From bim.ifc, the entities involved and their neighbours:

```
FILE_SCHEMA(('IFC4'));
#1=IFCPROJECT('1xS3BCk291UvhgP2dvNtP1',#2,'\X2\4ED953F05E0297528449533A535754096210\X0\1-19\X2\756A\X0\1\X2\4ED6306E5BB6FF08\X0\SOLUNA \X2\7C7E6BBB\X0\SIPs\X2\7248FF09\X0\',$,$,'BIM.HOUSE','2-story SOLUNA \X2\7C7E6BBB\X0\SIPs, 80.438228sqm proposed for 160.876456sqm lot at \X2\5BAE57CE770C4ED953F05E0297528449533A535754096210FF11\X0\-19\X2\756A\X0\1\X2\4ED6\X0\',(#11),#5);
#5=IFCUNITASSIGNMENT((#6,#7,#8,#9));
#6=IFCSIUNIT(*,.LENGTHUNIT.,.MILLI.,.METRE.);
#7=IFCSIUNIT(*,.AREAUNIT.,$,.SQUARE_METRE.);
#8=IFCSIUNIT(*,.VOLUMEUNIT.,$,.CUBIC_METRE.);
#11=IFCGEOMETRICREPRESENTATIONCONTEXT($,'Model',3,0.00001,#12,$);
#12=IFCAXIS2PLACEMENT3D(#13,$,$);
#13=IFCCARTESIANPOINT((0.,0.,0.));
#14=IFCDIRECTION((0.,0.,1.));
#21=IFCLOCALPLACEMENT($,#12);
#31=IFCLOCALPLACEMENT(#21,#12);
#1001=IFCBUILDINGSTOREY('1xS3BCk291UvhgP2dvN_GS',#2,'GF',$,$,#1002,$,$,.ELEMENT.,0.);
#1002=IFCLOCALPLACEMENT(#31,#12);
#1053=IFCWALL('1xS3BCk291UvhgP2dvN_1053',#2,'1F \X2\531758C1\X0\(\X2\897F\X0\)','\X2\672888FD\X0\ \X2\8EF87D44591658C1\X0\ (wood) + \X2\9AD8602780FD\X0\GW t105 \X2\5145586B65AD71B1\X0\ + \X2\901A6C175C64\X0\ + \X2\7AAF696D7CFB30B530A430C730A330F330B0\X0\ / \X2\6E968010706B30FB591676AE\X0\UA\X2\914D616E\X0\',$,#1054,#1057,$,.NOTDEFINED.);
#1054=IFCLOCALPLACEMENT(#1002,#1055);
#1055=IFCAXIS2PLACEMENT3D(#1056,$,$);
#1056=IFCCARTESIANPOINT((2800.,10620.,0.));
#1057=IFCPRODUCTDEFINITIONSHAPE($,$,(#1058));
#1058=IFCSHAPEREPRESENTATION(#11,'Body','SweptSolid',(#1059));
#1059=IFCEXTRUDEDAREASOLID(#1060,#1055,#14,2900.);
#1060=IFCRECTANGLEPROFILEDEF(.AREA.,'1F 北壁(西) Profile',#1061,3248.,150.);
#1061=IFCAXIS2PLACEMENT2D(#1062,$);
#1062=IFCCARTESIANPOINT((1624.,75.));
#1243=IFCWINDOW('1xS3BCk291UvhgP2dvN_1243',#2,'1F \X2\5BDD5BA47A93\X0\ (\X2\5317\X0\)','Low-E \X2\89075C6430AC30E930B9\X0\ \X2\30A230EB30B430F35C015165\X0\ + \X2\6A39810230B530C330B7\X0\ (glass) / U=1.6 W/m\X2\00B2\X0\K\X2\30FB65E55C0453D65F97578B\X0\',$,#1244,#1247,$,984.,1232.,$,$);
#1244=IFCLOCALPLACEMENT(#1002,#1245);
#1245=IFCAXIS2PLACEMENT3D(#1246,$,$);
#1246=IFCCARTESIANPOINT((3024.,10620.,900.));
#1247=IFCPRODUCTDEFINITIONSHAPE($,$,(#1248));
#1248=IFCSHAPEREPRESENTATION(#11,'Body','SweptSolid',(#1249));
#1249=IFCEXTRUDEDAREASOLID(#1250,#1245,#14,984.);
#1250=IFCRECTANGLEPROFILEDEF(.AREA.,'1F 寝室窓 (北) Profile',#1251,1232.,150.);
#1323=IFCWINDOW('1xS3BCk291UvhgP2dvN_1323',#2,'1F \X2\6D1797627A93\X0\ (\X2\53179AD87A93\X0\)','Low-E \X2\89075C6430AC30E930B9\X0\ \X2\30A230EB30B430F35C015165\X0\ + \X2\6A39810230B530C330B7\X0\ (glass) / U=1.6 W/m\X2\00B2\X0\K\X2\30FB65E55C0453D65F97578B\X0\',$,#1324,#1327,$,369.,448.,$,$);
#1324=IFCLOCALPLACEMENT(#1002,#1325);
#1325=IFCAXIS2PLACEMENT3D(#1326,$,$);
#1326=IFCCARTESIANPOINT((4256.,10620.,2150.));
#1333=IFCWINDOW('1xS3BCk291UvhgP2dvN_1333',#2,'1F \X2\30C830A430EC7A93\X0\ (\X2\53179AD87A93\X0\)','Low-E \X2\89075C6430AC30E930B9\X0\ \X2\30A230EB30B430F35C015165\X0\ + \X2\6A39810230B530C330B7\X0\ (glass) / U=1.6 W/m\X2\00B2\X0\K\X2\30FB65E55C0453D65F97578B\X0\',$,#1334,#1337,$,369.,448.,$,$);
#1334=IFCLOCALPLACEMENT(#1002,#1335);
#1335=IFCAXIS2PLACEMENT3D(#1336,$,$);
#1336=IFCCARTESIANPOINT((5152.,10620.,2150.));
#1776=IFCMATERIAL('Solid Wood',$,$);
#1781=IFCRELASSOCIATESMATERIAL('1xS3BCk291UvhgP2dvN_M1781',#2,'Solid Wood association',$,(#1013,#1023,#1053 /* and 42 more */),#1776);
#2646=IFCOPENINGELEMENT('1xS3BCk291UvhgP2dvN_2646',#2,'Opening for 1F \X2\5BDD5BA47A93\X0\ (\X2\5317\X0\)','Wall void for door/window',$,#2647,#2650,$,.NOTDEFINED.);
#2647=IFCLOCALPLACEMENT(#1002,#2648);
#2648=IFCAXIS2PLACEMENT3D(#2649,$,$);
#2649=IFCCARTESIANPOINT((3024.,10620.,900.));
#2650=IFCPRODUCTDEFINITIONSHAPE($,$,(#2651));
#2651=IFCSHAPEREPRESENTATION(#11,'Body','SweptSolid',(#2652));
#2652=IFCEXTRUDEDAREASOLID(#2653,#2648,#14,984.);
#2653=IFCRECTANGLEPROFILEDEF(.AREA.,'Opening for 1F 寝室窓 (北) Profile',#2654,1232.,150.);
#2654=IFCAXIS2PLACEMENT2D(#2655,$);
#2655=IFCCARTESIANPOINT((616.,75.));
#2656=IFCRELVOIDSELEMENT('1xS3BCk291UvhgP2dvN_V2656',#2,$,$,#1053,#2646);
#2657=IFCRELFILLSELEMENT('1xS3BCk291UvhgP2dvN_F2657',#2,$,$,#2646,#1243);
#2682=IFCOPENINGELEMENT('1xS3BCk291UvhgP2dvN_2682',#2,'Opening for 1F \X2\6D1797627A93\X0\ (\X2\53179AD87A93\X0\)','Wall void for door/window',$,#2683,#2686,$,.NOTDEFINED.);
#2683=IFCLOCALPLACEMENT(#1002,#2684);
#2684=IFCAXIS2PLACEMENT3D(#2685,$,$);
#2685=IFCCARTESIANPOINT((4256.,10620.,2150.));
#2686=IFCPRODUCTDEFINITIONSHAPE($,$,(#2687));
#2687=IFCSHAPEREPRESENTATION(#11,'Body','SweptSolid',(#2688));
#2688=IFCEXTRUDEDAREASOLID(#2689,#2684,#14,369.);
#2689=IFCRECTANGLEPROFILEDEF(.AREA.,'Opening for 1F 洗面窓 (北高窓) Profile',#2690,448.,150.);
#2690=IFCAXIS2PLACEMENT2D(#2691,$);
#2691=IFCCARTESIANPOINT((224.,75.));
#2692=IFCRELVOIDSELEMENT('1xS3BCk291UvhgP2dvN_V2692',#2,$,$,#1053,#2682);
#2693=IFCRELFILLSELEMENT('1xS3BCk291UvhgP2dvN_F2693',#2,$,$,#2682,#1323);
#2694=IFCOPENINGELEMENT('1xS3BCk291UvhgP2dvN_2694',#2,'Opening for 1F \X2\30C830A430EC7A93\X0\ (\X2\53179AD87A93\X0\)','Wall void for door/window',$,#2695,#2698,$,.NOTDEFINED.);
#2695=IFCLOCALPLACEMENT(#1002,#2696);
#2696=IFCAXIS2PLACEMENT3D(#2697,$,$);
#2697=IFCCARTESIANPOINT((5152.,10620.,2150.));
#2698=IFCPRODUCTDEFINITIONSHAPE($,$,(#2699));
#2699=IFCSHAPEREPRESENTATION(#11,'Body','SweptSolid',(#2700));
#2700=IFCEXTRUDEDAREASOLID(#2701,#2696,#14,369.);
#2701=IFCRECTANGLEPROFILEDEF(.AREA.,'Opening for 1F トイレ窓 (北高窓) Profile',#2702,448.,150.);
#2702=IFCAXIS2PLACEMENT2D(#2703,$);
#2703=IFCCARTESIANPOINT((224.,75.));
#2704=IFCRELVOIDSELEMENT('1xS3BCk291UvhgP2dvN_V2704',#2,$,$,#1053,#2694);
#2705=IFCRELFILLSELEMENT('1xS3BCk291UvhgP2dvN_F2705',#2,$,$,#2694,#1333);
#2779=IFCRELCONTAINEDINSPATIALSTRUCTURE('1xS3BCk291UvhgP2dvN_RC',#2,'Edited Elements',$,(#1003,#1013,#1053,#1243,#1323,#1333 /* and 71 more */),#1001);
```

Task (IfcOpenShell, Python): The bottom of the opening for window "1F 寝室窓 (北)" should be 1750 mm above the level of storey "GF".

```python
import numpy as np
import ifcopenshell
import ifcopenshell.api.geometry
import ifcopenshell.geom
import ifcopenshell.util.element
import ifcopenshell.util.placement
import ifcopenshell.util.shape
import ifcopenshell.util.unit

model = ifcopenshell.open("bim.ifc")
unit_scale = ifcopenshell.util.unit.calculate_unit_scale(model)

window = model.by_id(1243)
opening = window.FillsVoids[0].RelatingOpeningElement
storey = ifcopenshell.util.element.get_container(window, ifc_class="IfcBuildingStorey")
level = ifcopenshell.util.placement.get_local_placement(storey.ObjectPlacement)[2, 3]

# The opening's origin need not be at the sill, so measure its lowest point.
shape = ifcopenshell.geom.create_shape(ifcopenshell.geom.settings(), opening)
bottom = ifcopenshell.util.shape.get_shape_bottom_elevation(shape, shape.geometry) / unit_scale
dz = level + 1750.0 - bottom

shift = np.array([0.0, 0.0, dz])
# The window is not placed relative to its opening, so move both.
for product in (opening, window):
    matrix = ifcopenshell.util.placement.get_local_placement(product.ObjectPlacement)
    matrix[:3, 3] += shift
    ifcopenshell.api.geometry.edit_object_placement(model, product=product, matrix=matrix, is_si=False)

print(f"moved by {dz * unit_scale:+.3f} m")

model.write("bim_updated.ifc")
```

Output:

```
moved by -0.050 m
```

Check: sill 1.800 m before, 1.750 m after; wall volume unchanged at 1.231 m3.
